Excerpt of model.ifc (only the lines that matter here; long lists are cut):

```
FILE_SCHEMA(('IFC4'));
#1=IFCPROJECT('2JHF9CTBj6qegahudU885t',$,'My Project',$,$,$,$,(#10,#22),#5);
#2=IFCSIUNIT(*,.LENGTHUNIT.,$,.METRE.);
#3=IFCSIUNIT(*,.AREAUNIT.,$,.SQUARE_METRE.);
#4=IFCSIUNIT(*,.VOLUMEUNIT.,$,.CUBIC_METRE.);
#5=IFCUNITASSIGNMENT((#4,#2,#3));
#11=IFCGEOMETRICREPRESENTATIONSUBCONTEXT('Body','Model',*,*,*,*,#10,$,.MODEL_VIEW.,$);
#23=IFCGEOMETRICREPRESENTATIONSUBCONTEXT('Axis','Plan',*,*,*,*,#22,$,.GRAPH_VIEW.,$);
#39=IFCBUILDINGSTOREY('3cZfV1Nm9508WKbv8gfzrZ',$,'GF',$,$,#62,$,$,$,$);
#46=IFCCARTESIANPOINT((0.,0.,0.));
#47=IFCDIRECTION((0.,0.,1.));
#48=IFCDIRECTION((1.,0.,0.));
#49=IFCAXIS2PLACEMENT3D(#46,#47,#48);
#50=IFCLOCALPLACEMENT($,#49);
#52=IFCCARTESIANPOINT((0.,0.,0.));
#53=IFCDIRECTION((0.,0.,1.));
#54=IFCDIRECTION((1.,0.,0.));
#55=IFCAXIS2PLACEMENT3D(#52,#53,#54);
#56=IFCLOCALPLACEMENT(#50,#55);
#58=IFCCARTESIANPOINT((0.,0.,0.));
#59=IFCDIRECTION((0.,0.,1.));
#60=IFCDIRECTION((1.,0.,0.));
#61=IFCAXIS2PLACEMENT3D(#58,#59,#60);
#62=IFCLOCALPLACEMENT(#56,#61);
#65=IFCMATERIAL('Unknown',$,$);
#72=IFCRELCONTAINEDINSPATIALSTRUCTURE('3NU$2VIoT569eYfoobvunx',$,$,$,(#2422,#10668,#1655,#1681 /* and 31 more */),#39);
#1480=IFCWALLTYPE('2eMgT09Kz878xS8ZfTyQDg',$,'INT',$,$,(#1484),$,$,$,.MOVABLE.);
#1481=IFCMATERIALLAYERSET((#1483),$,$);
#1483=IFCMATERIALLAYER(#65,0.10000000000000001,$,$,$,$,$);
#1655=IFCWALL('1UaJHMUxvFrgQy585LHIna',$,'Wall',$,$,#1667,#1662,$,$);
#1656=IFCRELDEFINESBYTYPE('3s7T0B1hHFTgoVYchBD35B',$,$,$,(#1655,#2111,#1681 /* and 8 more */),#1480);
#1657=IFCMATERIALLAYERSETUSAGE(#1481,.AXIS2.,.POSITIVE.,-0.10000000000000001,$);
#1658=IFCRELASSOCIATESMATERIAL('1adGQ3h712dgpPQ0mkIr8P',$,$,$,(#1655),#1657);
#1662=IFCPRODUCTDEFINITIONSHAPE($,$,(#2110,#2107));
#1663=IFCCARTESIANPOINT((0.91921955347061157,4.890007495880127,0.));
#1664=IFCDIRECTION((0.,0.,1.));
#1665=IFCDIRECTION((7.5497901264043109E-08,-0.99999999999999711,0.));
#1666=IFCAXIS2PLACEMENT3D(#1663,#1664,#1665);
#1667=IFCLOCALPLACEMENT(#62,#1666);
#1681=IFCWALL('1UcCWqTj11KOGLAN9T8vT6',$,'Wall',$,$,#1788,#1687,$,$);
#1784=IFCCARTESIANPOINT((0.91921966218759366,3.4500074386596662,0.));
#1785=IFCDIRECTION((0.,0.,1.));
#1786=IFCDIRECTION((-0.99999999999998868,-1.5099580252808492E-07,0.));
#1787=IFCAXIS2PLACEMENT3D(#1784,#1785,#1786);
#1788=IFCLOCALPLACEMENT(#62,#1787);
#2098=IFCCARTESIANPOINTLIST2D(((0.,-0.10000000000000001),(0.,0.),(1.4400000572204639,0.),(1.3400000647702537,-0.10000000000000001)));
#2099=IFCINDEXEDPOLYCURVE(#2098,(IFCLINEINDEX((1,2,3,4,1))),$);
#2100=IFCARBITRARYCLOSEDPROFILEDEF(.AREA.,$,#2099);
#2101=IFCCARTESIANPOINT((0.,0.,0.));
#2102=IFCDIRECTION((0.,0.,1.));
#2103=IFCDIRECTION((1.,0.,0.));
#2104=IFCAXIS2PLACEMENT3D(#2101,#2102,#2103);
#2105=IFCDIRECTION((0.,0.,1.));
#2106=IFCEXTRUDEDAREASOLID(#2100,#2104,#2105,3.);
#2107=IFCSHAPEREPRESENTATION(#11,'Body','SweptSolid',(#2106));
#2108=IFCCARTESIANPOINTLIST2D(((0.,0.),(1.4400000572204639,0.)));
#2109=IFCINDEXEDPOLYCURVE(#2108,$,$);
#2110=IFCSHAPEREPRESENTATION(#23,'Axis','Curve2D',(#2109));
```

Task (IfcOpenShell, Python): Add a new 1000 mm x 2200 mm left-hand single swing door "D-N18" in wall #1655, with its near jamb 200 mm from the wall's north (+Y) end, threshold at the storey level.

```python
import numpy as np
import ifcopenshell
import ifcopenshell.api.feature
import ifcopenshell.api.geometry
import ifcopenshell.api.root
import ifcopenshell.api.spatial
import ifcopenshell.geom
import ifcopenshell.util.element
import ifcopenshell.util.placement
import ifcopenshell.util.representation
import ifcopenshell.util.shape
import ifcopenshell.util.unit

model = ifcopenshell.open("model.ifc")
unit_scale = ifcopenshell.util.unit.calculate_unit_scale(model)
settings = ifcopenshell.geom.settings()


def volume(element):
    """Net volume in cubic metres, openings subtracted."""
    shape = ifcopenshell.geom.create_shape(settings, element)
    return ifcopenshell.util.shape.get_volume(shape.geometry)


wall = model.by_guid("1UaJHMUxvFrgQy585LHIna")
storey = ifcopenshell.util.element.get_container(wall, ifc_class="IfcBuildingStorey")
context = ifcopenshell.util.representation.get_context(model, "Model", "Body", "MODEL_VIEW")
before = volume(wall)

width, height, from_end, sill = 1, 2.2, 0.2, 0.0  # metres

# The wall runs along its own X axis, and the end named is its -X end.
wall_shape = ifcopenshell.geom.create_shape(settings, wall)
x, y, z = ifcopenshell.util.shape.get_vertices(wall_shape.geometry).T
start = x.min() + from_end
face, thickness = float(y.min()), float(y.max() - y.min())
wall_matrix = ifcopenshell.util.placement.get_local_placement(wall.ObjectPlacement)
level = ifcopenshell.util.placement.get_local_placement(storey.ObjectPlacement)[2, 3]


def in_wall(x, y):
    """Placement at x, y metres in the wall's axes, at sill height."""
    matrix = wall_matrix.copy()
    matrix[:, 3] = wall_matrix @ np.array([x / unit_scale, y / unit_scale, 0.0, 1.0])
    matrix[2, 3] = level + sill / unit_scale
    return matrix


# Opening: a box that overshoots both wall faces by 50 mm.
opening = ifcopenshell.api.root.create_entity(model, ifc_class="IfcOpeningElement", predefined_type="OPENING")
box = ifcopenshell.api.geometry.add_wall_representation(
    model, context=context, length=width, height=height, thickness=thickness + 0.1
)
ifcopenshell.api.geometry.assign_representation(model, product=opening, representation=box)
ifcopenshell.api.geometry.edit_object_placement(model, product=opening, matrix=in_wall(start, face - 0.05), is_si=False)
ifcopenshell.api.feature.add_feature(model, feature=opening, element=wall)

door = ifcopenshell.api.root.create_entity(model, ifc_class="IfcDoor", name="D-N18", predefined_type="DOOR")
door.OverallWidth, door.OverallHeight = width / unit_scale, height / unit_scale
door.OperationType = "SINGLE_SWING_LEFT"
body = ifcopenshell.api.geometry.add_door_representation(
    model,
    context=context,
    overall_width=door.OverallWidth,
    overall_height=door.OverallHeight,
    operation_type="SINGLE_SWING_LEFT",
    lining_properties={"LiningDepth": thickness / unit_scale, "ThresholdDepth": thickness / unit_scale},
)
ifcopenshell.api.geometry.assign_representation(model, product=door, representation=body)
ifcopenshell.api.spatial.assign_container(model, products=[door], relating_structure=storey)
ifcopenshell.api.feature.add_filling(model, opening=opening, element=door)

# The lining spans the wall, so the door starts at the wall face.
ifcopenshell.api.geometry.edit_object_placement(model, product=door, matrix=in_wall(start, face), is_si=False)

after = volume(wall)

print(f"wall volume {before:.3f} -> {after:.3f} m3")

model.write("model_rev.ifc")
```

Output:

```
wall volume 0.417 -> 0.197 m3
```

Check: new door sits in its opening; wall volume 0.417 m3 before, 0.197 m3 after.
